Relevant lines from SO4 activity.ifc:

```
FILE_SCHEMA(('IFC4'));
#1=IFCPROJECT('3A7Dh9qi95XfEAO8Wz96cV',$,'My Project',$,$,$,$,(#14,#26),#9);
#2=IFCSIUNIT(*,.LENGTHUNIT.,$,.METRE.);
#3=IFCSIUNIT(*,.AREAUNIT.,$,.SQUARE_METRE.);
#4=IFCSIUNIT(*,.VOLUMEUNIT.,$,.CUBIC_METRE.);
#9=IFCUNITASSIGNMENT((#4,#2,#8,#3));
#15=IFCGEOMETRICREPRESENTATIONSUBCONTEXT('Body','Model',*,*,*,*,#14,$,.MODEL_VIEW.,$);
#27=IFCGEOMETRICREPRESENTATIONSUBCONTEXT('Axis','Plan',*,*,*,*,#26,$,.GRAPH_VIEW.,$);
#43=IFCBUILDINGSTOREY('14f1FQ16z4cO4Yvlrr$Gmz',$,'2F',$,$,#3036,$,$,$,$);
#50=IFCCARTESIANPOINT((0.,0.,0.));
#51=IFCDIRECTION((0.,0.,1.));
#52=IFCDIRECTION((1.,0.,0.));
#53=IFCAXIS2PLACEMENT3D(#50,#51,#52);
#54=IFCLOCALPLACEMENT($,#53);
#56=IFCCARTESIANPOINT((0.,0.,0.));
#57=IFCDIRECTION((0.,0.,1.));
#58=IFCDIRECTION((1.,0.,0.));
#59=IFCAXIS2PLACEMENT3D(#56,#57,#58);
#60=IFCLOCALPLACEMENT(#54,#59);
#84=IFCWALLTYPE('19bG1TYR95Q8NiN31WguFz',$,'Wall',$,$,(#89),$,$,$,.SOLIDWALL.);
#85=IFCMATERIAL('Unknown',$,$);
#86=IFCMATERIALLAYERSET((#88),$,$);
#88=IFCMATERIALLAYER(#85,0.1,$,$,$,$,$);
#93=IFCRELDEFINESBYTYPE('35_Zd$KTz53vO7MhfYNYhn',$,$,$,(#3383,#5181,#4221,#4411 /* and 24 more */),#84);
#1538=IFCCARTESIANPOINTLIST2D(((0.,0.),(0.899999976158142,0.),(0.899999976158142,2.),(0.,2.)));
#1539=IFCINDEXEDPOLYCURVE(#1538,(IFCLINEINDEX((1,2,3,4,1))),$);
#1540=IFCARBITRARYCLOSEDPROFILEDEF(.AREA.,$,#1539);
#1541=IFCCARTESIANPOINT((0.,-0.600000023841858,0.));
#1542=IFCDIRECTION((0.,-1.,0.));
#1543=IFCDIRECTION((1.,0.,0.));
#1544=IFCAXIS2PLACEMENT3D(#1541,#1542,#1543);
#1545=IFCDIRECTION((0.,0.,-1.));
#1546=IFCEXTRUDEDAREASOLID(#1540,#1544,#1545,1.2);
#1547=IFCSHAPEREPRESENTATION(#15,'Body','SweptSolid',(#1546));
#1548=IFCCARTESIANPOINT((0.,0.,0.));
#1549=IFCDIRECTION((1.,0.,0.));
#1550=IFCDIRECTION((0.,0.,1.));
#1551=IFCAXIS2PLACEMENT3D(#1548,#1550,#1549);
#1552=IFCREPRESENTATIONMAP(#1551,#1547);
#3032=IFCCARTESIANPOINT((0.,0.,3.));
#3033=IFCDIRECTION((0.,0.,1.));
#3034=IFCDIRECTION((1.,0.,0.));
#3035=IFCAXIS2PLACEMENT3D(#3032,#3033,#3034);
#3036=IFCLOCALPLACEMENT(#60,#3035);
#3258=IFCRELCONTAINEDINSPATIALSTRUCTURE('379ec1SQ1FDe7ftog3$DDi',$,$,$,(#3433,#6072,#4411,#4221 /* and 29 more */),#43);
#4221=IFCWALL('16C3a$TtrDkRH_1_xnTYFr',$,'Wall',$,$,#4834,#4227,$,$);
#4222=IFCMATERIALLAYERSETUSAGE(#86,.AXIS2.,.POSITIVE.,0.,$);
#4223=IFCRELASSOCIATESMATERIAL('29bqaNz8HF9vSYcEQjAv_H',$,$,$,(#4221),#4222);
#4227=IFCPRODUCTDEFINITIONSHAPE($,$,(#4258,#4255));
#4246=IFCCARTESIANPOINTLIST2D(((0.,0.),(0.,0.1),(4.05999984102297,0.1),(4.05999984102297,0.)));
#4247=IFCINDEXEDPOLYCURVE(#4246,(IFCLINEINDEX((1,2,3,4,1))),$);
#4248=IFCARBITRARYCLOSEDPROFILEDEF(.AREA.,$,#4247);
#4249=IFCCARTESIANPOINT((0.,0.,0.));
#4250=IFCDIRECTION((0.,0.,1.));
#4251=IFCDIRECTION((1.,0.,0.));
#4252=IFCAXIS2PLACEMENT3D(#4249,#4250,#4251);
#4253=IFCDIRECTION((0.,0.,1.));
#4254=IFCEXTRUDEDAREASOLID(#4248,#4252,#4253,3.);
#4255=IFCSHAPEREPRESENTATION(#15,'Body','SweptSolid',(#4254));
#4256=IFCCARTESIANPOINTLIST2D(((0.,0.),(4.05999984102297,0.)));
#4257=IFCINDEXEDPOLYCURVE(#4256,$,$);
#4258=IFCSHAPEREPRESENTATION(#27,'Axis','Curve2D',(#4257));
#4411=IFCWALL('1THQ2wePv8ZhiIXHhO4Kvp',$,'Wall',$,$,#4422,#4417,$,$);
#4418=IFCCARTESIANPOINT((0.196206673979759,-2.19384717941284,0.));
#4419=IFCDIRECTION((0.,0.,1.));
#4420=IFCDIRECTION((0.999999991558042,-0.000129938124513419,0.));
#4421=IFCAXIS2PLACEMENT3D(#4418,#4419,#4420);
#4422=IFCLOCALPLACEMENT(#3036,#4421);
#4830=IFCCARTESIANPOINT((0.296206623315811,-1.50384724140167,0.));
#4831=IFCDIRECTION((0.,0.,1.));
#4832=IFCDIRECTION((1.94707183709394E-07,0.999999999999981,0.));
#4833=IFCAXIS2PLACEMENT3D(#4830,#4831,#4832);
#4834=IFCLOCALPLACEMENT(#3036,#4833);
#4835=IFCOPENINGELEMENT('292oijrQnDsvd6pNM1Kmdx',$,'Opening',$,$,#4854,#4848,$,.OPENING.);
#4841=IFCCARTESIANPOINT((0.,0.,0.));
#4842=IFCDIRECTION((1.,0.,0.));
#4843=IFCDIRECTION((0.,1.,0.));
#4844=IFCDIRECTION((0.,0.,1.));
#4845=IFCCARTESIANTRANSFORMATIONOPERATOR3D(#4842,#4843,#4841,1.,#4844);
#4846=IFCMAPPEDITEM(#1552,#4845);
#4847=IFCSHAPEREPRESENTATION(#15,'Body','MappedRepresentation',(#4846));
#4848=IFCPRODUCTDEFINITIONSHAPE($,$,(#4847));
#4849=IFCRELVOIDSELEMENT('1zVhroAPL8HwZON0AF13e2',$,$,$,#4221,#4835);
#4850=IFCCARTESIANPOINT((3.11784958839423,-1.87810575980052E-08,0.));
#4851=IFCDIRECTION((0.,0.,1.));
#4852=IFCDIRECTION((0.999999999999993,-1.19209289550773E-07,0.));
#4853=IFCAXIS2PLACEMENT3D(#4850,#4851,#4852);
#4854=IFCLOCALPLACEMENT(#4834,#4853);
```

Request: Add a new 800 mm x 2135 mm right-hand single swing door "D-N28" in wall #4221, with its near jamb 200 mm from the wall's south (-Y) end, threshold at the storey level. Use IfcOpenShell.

```python
import numpy as np
import ifcopenshell
import ifcopenshell.api.feature
import ifcopenshell.api.geometry
import ifcopenshell.api.root
import ifcopenshell.api.spatial
import ifcopenshell.geom
import ifcopenshell.util.element
import ifcopenshell.util.placement
import ifcopenshell.util.representation
import ifcopenshell.util.shape
import ifcopenshell.util.unit

model = ifcopenshell.open("SO4 activity.ifc")
unit_scale = ifcopenshell.util.unit.calculate_unit_scale(model)
settings = ifcopenshell.geom.settings()


def volume(element):
    """Net volume in cubic metres, openings subtracted."""
    shape = ifcopenshell.geom.create_shape(settings, element)
    return ifcopenshell.util.shape.get_volume(shape.geometry)


wall = model.by_id(4221)
storey = ifcopenshell.util.element.get_container(wall, ifc_class="IfcBuildingStorey")
context = ifcopenshell.util.representation.get_context(model, "Model", "Body", "MODEL_VIEW")
before = volume(wall)

width, height, from_end, sill = 0.8, 2.135, 0.2, 0.0  # metres

# The wall runs along its own X axis, and the end named is its -X end.
wall_shape = ifcopenshell.geom.create_shape(settings, wall)
x, y, z = ifcopenshell.util.shape.get_vertices(wall_shape.geometry).T
start = x.min() + from_end
face, thickness = float(y.min()), float(y.max() - y.min())
wall_matrix = ifcopenshell.util.placement.get_local_placement(wall.ObjectPlacement)
level = ifcopenshell.util.placement.get_local_placement(storey.ObjectPlacement)[2, 3]


def in_wall(x, y):
    """Placement at x, y metres in the wall's axes, at sill height."""
    matrix = wall_matrix.copy()
    matrix[:, 3] = wall_matrix @ np.array([x / unit_scale, y / unit_scale, 0.0, 1.0])
    matrix[2, 3] = level + sill / unit_scale
    return matrix


# Opening: a box that overshoots both wall faces by 50 mm.
opening = ifcopenshell.api.root.create_entity(model, ifc_class="IfcOpeningElement", predefined_type="OPENING")
box = ifcopenshell.api.geometry.add_wall_representation(
    model, context=context, length=width, height=height, thickness=thickness + 0.1
)
ifcopenshell.api.geometry.assign_representation(model, product=opening, representation=box)
ifcopenshell.api.geometry.edit_object_placement(model, product=opening, matrix=in_wall(start, face - 0.05), is_si=False)
ifcopenshell.api.feature.add_feature(model, feature=opening, element=wall)

door = ifcopenshell.api.root.create_entity(model, ifc_class="IfcDoor", name="D-N28", predefined_type="DOOR")
door.OverallWidth, door.OverallHeight = width / unit_scale, height / unit_scale
door.OperationType = "SINGLE_SWING_RIGHT"
body = ifcopenshell.api.geometry.add_door_representation(
    model,
    context=context,
    overall_width=door.OverallWidth,
    overall_height=door.OverallHeight,
    operation_type="SINGLE_SWING_RIGHT",
    lining_properties={"LiningDepth": thickness / unit_scale, "ThresholdDepth": thickness / unit_scale},
)
ifcopenshell.api.geometry.assign_representation(model, product=door, representation=body)
ifcopenshell.api.spatial.assign_container(model, products=[door], relating_structure=storey)
ifcopenshell.api.feature.add_filling(model, opening=opening, element=door)

# The lining spans the wall, so the door starts at the wall face.
ifcopenshell.api.geometry.edit_object_placement(model, product=door, matrix=in_wall(start, face), is_si=False)

after = volume(wall)

print(f"wall volume {before:.3f} -> {after:.3f} m3")

model.write("SO4 activity_edited.ifc")
```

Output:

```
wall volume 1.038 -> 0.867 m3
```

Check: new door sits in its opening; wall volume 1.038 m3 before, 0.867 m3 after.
